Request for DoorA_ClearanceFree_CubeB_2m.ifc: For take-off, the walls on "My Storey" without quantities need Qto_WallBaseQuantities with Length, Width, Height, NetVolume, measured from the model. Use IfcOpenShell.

First a look at what the model holds.

```python
import ifcopenshell
import ifcopenshell.util.element
import ifcopenshell.util.unit

model = ifcopenshell.open("DoorA_ClearanceFree_CubeB_2m.ifc")
print(model.schema)
for unit_type in ("LENGTHUNIT", "AREAUNIT", "VOLUMEUNIT"):
    print(unit_type, ifcopenshell.util.unit.calculate_unit_scale(model, unit_type))
storey = next(s for s in model.by_type("IfcBuildingStorey") if s.Name == "My Storey")
walls = [e for e in ifcopenshell.util.element.get_decomposition(storey) if e.is_a("IfcWall")]
for e in sorted(walls, key=lambda e: e.id()):
    print(e.id(), e.is_a(), e.Name, list(ifcopenshell.util.element.get_psets(e, qtos_only=True)), sep=" | ")
```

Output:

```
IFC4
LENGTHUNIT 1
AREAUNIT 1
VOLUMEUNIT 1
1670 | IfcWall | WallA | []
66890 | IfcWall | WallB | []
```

```python
import ifcopenshell
import ifcopenshell.api.pset
import ifcopenshell.geom
import ifcopenshell.util.element
import ifcopenshell.util.shape
import ifcopenshell.util.unit

model = ifcopenshell.open("DoorA_ClearanceFree_CubeB_2m.ifc")
unit_scale = ifcopenshell.util.unit.calculate_unit_scale(model)
volume_scale = ifcopenshell.util.unit.calculate_unit_scale(model, "VOLUMEUNIT")
settings = ifcopenshell.geom.settings()

storey = next(s for s in model.by_type("IfcBuildingStorey") if s.Name == "My Storey")
walls = [e for e in ifcopenshell.util.element.get_decomposition(storey) if e.is_a("IfcWall")]

for e in sorted(walls, key=lambda e: e.id()):
    if ifcopenshell.util.element.get_psets(e, qtos_only=True, should_inherit=False):
        continue
    # Geometry comes back in metres, in the element's own axes.
    shape = ifcopenshell.geom.create_shape(settings, e)
    values = {
        "Length": ifcopenshell.util.shape.get_x(shape.geometry) / unit_scale,
        "Width": ifcopenshell.util.shape.get_y(shape.geometry) / unit_scale,
        "Height": ifcopenshell.util.shape.get_z(shape.geometry) / unit_scale,
        "NetVolume": ifcopenshell.util.shape.get_volume(shape.geometry) / volume_scale,
    }
    qto = ifcopenshell.api.pset.add_qto(model, product=e, name="Qto_WallBaseQuantities")
    ifcopenshell.api.pset.edit_qto(model, qto=qto, properties=values)
    print(e.id(), {k: round(v, 3) for k, v in values.items()})

model.write("DoorA_ClearanceFree_CubeB_2m-out.ifc")
```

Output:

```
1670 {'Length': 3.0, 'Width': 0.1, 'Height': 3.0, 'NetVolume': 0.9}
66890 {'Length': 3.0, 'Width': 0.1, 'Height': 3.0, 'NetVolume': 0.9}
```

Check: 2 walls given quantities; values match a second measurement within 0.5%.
